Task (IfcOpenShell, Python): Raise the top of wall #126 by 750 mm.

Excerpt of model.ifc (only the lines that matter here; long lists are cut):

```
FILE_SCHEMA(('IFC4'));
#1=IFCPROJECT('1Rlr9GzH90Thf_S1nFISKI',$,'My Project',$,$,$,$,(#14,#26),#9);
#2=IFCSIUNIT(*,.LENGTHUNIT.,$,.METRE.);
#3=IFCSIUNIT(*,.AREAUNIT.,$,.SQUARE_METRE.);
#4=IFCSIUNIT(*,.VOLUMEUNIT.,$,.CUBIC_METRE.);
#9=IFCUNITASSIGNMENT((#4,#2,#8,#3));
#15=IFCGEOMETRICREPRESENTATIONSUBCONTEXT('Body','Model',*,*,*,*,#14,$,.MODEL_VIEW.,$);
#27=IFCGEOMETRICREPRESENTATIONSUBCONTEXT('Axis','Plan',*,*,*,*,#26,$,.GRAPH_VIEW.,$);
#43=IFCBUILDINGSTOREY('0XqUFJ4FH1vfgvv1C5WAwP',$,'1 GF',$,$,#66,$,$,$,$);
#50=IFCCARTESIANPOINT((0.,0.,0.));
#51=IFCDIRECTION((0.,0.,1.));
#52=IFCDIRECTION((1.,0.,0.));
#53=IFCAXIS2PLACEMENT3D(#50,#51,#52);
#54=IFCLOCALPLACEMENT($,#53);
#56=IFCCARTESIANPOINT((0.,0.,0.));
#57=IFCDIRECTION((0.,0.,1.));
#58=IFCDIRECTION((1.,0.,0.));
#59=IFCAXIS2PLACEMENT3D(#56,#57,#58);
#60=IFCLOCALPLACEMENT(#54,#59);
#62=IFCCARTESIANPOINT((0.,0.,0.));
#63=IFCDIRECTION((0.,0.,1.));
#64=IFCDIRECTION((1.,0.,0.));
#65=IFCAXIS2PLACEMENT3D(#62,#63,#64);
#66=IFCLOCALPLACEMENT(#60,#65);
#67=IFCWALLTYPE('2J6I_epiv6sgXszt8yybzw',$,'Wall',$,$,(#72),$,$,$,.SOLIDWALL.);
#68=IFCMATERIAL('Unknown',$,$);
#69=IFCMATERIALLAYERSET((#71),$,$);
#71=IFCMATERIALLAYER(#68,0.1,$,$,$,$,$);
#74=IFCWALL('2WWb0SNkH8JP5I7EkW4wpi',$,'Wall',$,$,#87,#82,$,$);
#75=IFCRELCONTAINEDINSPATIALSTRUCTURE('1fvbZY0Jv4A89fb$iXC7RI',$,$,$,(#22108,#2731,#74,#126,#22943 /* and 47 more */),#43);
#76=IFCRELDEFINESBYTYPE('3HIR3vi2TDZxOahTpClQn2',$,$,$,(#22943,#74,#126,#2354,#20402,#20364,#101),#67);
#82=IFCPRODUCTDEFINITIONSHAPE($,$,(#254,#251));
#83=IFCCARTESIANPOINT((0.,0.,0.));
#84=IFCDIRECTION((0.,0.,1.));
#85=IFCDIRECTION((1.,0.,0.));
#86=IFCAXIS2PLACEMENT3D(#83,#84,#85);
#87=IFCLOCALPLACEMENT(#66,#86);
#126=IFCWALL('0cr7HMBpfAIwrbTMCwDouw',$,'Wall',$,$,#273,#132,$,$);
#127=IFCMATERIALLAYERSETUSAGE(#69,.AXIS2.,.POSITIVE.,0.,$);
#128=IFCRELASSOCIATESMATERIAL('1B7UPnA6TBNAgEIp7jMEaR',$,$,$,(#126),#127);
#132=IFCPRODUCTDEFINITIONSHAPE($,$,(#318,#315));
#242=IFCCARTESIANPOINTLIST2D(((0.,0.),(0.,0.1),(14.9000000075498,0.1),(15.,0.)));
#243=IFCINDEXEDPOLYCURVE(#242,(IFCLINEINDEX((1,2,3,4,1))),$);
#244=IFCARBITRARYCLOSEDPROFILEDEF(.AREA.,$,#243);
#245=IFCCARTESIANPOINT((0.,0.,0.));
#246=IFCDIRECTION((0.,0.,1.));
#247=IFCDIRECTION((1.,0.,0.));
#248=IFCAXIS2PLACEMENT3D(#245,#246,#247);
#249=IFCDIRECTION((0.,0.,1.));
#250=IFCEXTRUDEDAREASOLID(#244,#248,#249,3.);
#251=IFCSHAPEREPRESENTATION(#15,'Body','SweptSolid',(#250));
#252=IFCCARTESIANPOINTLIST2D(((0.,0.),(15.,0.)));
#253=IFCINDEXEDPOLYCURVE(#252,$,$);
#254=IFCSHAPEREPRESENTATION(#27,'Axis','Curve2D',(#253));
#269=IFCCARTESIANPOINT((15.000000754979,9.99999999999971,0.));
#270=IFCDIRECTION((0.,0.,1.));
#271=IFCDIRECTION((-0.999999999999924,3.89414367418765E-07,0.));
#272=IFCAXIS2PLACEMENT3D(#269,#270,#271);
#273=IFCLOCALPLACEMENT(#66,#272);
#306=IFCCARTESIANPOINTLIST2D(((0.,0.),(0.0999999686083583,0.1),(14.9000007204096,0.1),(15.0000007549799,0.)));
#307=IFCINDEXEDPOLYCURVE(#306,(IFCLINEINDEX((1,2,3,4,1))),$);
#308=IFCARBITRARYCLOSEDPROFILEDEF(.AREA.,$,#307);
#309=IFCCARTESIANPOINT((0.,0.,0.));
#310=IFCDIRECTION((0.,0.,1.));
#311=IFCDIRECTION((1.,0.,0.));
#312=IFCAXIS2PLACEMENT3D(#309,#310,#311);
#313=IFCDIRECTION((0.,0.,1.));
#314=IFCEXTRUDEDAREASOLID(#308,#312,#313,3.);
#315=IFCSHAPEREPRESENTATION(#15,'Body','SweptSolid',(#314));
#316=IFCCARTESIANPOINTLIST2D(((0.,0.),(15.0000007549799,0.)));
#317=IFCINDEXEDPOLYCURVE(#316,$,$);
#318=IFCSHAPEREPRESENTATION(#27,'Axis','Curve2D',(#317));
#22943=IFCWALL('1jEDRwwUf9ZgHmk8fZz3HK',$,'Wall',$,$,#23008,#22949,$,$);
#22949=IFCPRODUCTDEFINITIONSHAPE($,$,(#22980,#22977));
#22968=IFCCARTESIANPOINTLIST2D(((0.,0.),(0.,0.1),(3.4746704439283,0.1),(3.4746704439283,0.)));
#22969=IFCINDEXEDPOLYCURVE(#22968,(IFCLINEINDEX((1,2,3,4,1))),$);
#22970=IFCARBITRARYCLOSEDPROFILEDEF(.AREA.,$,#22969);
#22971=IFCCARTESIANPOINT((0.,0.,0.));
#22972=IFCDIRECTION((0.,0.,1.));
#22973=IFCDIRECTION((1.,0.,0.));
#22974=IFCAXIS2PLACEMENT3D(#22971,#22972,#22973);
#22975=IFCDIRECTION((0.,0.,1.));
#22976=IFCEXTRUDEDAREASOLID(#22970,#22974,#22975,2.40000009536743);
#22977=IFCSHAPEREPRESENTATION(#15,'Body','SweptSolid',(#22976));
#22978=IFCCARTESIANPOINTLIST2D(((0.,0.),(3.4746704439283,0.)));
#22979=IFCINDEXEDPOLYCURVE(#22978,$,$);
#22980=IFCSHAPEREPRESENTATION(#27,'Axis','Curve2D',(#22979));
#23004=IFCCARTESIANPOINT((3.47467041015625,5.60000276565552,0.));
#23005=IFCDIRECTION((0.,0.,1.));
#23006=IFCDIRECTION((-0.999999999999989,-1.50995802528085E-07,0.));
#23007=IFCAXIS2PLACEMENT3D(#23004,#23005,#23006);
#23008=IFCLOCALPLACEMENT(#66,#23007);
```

```python
import ifcopenshell
import ifcopenshell.geom
import ifcopenshell.util.representation
import ifcopenshell.util.shape
import ifcopenshell.util.unit

model = ifcopenshell.open("model.ifc")
unit_scale = ifcopenshell.util.unit.calculate_unit_scale(model)
settings = ifcopenshell.geom.settings()


def volume(element):
    """Net volume in cubic metres, openings subtracted."""
    shape = ifcopenshell.geom.create_shape(settings, element)
    return ifcopenshell.util.shape.get_volume(shape.geometry)


wall = model.by_guid("0cr7HMBpfAIwrbTMCwDouw")
before = volume(wall)

body = ifcopenshell.util.representation.get_representation(wall, "Model", "Body")
solid = body.Items[0]
old_height = solid.Depth
solid.Depth += 0.75 / unit_scale
after = volume(wall)

print(f"height {old_height:g} -> {solid.Depth:g}, volume {before:.3f} -> {after:.3f} m3")

model.write("model_rev.ifc")
```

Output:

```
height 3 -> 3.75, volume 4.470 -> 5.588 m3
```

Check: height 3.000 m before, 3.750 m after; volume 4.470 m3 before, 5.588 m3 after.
